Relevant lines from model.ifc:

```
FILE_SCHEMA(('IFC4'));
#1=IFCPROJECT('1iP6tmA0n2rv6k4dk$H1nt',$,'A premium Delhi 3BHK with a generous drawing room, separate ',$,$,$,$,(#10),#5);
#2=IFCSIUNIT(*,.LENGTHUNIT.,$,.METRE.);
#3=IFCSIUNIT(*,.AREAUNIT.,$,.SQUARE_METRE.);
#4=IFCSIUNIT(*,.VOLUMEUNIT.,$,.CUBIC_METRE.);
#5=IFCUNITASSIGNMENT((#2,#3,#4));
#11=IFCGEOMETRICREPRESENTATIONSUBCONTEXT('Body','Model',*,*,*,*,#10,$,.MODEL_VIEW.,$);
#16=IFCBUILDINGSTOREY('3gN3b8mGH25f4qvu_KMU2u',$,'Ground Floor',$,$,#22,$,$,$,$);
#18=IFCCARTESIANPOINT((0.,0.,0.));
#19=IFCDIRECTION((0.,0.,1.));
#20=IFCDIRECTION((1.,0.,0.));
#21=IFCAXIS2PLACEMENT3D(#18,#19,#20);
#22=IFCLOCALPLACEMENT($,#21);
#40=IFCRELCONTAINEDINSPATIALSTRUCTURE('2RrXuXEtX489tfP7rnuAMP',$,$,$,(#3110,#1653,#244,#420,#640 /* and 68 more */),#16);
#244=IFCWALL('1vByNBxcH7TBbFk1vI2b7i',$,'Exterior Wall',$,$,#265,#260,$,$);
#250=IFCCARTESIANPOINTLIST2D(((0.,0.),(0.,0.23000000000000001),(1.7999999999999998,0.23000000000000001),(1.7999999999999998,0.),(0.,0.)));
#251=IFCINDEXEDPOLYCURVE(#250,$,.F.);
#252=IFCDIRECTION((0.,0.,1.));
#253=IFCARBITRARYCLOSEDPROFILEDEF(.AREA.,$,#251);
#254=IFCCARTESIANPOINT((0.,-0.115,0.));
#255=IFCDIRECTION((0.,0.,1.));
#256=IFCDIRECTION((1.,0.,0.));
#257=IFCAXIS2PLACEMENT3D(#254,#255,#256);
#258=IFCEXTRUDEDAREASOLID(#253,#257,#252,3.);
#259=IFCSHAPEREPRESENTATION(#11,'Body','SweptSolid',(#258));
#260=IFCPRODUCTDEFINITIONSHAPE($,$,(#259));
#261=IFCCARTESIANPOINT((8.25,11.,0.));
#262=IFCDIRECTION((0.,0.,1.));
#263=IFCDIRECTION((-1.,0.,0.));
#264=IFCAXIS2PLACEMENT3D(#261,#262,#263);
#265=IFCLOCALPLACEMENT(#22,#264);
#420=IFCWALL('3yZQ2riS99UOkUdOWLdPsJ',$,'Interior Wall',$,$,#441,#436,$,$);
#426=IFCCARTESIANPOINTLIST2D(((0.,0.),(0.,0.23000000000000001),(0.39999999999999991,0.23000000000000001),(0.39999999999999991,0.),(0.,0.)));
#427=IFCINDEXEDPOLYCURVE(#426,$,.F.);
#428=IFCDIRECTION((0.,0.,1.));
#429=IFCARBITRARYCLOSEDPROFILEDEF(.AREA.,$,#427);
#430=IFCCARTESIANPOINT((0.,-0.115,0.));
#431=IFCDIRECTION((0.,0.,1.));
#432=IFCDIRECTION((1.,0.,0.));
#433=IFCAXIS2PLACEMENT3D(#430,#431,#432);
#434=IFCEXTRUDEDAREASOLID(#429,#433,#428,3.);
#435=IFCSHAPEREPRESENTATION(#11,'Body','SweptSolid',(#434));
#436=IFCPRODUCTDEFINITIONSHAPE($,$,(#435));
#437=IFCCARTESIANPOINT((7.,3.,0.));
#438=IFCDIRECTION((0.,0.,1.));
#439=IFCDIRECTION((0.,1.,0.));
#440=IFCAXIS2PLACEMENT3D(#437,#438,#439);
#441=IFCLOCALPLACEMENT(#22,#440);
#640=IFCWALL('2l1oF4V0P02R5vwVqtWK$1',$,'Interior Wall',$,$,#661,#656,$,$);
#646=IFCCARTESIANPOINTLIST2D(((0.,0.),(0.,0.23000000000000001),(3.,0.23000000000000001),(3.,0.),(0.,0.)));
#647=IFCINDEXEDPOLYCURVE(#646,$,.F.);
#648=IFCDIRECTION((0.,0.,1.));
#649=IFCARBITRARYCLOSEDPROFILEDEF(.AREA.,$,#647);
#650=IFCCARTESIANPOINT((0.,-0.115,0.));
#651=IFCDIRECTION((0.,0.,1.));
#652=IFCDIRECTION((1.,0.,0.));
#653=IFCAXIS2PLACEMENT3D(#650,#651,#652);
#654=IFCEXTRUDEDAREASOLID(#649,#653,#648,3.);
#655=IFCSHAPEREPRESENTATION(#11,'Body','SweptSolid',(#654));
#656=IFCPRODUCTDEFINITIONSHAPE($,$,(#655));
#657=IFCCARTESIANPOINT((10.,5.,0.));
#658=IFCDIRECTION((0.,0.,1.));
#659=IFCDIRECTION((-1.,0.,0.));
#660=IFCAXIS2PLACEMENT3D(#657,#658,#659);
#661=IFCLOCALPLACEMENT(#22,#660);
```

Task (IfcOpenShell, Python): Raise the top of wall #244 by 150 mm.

```python
import ifcopenshell
import ifcopenshell.geom
import ifcopenshell.util.representation
import ifcopenshell.util.shape
import ifcopenshell.util.unit

model = ifcopenshell.open("model.ifc")
unit_scale = ifcopenshell.util.unit.calculate_unit_scale(model)
settings = ifcopenshell.geom.settings()


def volume(element):
    """Net volume in cubic metres, openings subtracted."""
    shape = ifcopenshell.geom.create_shape(settings, element)
    return ifcopenshell.util.shape.get_volume(shape.geometry)


wall = model.by_guid("1vByNBxcH7TBbFk1vI2b7i")
before = volume(wall)

body = ifcopenshell.util.representation.get_representation(wall, "Model", "Body")
solid = body.Items[0]
old_height = solid.Depth
solid.Depth += 0.15 / unit_scale
after = volume(wall)

print(f"height {old_height:g} -> {solid.Depth:g}, volume {before:.3f} -> {after:.3f} m3")

model.write("model-out.ifc")
```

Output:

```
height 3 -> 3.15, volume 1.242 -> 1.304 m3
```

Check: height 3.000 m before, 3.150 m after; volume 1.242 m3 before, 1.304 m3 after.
